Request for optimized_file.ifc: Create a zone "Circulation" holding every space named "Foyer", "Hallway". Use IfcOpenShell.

First a look at what the model holds.

```python
import ifcopenshell

model = ifcopenshell.open("optimized_file.ifc")
print(model.schema)
seen = {}
for space in model.by_type("IfcSpace"):
    seen[space.LongName] = seen.get(space.LongName, 0) + 1
for name, count in sorted(seen.items(), key=str):
    print(count, "x", name)
print("zones:", [z.Name for z in model.by_type("IfcZone")][:20])
```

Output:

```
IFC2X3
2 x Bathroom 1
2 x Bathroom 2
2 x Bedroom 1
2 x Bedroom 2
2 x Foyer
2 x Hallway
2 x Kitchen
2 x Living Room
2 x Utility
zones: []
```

```python
import ifcopenshell
import ifcopenshell.api.group
import ifcopenshell.api.root

model = ifcopenshell.open("optimized_file.ifc")

names = {"Foyer", "Hallway"}
spaces = [s for s in model.by_type("IfcSpace") if s.LongName in names]

zone = ifcopenshell.api.root.create_entity(model, ifc_class="IfcZone", name="Circulation")
ifcopenshell.api.group.assign_group(model, products=spaces, group=zone)
print(len(spaces), "spaces in", zone.Name)

model.write("optimized_file_v2.ifc")
```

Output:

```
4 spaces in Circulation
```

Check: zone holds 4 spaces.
